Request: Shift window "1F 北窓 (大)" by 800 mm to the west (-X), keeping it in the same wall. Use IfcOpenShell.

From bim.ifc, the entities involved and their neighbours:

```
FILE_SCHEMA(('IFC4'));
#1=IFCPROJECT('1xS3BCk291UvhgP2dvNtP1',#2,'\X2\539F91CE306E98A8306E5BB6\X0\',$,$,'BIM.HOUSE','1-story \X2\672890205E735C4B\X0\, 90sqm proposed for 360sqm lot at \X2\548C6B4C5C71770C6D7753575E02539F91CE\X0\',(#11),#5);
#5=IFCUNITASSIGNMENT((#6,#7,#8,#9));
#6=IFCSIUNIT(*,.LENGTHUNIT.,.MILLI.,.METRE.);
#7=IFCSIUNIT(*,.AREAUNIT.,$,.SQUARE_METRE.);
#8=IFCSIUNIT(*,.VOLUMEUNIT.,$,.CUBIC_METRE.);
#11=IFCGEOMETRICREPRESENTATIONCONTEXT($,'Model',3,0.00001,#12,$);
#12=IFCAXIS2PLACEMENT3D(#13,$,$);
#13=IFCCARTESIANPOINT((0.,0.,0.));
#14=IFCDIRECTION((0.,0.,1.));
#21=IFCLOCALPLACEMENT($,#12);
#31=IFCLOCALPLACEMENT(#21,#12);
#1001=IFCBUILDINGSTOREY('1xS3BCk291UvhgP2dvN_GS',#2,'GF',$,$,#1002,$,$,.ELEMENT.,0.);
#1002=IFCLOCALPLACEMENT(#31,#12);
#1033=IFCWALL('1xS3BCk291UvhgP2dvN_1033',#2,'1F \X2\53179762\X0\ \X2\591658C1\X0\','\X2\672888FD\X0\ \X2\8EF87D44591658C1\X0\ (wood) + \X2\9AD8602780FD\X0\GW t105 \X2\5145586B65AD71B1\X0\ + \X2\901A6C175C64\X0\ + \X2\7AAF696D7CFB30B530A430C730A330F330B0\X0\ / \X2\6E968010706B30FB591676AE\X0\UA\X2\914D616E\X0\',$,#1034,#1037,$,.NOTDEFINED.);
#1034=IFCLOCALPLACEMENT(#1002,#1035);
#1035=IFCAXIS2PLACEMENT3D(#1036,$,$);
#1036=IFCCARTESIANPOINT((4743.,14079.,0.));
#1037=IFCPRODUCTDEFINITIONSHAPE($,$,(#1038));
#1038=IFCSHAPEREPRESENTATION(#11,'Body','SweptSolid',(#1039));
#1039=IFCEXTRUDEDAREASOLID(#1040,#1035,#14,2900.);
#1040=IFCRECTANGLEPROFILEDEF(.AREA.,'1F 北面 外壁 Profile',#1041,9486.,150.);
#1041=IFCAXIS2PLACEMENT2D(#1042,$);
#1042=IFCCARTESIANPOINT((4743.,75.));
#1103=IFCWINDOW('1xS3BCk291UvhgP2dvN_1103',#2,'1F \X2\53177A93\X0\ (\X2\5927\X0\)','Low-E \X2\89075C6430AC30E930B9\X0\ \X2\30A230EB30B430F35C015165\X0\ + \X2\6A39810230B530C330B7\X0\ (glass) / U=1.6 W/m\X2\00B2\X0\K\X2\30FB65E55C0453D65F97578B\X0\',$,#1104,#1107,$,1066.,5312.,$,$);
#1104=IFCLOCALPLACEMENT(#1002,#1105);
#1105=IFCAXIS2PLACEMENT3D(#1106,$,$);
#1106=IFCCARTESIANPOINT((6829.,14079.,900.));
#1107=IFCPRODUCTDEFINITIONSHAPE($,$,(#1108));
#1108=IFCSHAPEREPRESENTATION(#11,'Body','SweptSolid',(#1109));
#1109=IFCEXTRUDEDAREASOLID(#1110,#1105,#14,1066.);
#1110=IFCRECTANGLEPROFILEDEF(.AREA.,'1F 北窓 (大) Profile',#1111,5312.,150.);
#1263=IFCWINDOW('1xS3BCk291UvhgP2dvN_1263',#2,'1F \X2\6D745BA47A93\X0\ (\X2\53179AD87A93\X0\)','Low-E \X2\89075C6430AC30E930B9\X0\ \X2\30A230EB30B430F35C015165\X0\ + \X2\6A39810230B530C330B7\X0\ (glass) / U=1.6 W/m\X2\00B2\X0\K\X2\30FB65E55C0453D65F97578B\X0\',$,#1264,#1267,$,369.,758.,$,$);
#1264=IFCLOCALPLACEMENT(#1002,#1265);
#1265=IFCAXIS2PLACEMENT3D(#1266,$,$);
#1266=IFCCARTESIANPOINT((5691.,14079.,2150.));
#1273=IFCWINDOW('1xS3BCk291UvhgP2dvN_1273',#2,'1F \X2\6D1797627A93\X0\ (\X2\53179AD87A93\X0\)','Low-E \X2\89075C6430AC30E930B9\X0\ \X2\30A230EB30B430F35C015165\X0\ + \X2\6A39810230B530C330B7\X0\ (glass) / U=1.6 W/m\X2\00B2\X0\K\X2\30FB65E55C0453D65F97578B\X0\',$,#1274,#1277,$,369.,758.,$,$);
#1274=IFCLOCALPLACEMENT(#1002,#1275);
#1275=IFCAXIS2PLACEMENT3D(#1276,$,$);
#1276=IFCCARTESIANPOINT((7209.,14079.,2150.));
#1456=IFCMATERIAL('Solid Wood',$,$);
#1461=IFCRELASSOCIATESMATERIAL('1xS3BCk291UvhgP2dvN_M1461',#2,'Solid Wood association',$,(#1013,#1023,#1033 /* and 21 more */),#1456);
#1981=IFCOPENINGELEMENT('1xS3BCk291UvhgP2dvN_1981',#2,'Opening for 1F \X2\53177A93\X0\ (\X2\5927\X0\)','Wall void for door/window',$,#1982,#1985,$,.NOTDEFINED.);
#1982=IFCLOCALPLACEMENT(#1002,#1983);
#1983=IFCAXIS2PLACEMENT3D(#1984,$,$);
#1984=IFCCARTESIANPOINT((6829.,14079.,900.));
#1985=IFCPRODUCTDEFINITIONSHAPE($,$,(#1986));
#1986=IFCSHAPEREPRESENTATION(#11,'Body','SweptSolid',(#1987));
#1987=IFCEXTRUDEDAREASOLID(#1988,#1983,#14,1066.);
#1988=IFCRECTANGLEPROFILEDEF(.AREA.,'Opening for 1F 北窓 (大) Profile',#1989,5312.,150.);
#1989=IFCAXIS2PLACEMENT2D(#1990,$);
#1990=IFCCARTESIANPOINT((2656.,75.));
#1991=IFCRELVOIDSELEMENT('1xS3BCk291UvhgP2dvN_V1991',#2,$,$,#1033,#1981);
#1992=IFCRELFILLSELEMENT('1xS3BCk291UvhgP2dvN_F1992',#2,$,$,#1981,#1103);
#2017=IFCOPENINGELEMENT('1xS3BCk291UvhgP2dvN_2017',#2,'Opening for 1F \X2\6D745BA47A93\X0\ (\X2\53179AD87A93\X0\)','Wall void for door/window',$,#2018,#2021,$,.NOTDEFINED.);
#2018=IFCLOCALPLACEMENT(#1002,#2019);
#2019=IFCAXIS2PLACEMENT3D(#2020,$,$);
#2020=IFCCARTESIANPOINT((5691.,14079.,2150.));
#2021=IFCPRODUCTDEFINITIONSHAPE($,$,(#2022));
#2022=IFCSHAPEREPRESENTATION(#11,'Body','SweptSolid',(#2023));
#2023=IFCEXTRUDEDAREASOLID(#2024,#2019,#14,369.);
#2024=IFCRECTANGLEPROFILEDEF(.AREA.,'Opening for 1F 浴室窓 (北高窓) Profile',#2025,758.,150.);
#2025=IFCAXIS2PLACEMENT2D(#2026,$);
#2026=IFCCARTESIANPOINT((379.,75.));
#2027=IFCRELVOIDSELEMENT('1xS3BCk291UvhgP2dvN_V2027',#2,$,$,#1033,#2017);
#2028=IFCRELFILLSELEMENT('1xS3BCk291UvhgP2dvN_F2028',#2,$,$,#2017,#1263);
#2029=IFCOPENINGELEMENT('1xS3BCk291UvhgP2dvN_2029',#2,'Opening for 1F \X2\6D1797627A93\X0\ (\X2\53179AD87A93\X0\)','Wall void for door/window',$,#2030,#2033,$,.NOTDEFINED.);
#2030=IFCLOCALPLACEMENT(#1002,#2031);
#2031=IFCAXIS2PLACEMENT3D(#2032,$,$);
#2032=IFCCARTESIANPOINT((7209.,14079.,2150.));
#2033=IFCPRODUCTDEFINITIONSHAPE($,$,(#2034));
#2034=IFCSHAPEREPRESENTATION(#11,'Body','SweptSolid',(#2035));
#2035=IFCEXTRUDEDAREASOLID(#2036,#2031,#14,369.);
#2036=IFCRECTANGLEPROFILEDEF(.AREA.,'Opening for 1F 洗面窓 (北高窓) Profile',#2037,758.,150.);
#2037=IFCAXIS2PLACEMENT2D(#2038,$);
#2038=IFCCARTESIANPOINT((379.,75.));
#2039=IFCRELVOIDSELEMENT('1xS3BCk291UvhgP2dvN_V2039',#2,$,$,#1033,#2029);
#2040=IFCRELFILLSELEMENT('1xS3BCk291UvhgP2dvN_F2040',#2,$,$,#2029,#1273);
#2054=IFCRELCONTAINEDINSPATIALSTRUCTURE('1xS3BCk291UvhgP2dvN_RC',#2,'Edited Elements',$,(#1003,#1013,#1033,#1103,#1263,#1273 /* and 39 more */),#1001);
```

```python
import ifcopenshell
import ifcopenshell.api.geometry
import ifcopenshell.util.placement
import ifcopenshell.util.unit

model = ifcopenshell.open("bim.ifc")
unit_scale = ifcopenshell.util.unit.calculate_unit_scale(model)

window = model.by_id(1103)
opening = window.FillsVoids[0].RelatingOpeningElement
wall = opening.VoidsElements[0].RelatingBuildingElement

wall_matrix = ifcopenshell.util.placement.get_local_placement(wall.ObjectPlacement)
shift = wall_matrix[:3, 0] * -0.8 / unit_scale
before = ifcopenshell.util.placement.get_local_placement(window.ObjectPlacement)[:3, 3].copy()

# The window is not placed relative to its opening, so move both.
for product in (opening, window):
    matrix = ifcopenshell.util.placement.get_local_placement(product.ObjectPlacement)
    matrix[:3, 3] += shift
    ifcopenshell.api.geometry.edit_object_placement(model, product=product, matrix=matrix, is_si=False)

after = ifcopenshell.util.placement.get_local_placement(window.ObjectPlacement)[:3, 3]
print("window moved by", (after - before).round(3) + 0.0)

model.write("bim_v2.ifc")
```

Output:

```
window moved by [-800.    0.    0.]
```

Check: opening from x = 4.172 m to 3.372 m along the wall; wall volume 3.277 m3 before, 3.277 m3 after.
